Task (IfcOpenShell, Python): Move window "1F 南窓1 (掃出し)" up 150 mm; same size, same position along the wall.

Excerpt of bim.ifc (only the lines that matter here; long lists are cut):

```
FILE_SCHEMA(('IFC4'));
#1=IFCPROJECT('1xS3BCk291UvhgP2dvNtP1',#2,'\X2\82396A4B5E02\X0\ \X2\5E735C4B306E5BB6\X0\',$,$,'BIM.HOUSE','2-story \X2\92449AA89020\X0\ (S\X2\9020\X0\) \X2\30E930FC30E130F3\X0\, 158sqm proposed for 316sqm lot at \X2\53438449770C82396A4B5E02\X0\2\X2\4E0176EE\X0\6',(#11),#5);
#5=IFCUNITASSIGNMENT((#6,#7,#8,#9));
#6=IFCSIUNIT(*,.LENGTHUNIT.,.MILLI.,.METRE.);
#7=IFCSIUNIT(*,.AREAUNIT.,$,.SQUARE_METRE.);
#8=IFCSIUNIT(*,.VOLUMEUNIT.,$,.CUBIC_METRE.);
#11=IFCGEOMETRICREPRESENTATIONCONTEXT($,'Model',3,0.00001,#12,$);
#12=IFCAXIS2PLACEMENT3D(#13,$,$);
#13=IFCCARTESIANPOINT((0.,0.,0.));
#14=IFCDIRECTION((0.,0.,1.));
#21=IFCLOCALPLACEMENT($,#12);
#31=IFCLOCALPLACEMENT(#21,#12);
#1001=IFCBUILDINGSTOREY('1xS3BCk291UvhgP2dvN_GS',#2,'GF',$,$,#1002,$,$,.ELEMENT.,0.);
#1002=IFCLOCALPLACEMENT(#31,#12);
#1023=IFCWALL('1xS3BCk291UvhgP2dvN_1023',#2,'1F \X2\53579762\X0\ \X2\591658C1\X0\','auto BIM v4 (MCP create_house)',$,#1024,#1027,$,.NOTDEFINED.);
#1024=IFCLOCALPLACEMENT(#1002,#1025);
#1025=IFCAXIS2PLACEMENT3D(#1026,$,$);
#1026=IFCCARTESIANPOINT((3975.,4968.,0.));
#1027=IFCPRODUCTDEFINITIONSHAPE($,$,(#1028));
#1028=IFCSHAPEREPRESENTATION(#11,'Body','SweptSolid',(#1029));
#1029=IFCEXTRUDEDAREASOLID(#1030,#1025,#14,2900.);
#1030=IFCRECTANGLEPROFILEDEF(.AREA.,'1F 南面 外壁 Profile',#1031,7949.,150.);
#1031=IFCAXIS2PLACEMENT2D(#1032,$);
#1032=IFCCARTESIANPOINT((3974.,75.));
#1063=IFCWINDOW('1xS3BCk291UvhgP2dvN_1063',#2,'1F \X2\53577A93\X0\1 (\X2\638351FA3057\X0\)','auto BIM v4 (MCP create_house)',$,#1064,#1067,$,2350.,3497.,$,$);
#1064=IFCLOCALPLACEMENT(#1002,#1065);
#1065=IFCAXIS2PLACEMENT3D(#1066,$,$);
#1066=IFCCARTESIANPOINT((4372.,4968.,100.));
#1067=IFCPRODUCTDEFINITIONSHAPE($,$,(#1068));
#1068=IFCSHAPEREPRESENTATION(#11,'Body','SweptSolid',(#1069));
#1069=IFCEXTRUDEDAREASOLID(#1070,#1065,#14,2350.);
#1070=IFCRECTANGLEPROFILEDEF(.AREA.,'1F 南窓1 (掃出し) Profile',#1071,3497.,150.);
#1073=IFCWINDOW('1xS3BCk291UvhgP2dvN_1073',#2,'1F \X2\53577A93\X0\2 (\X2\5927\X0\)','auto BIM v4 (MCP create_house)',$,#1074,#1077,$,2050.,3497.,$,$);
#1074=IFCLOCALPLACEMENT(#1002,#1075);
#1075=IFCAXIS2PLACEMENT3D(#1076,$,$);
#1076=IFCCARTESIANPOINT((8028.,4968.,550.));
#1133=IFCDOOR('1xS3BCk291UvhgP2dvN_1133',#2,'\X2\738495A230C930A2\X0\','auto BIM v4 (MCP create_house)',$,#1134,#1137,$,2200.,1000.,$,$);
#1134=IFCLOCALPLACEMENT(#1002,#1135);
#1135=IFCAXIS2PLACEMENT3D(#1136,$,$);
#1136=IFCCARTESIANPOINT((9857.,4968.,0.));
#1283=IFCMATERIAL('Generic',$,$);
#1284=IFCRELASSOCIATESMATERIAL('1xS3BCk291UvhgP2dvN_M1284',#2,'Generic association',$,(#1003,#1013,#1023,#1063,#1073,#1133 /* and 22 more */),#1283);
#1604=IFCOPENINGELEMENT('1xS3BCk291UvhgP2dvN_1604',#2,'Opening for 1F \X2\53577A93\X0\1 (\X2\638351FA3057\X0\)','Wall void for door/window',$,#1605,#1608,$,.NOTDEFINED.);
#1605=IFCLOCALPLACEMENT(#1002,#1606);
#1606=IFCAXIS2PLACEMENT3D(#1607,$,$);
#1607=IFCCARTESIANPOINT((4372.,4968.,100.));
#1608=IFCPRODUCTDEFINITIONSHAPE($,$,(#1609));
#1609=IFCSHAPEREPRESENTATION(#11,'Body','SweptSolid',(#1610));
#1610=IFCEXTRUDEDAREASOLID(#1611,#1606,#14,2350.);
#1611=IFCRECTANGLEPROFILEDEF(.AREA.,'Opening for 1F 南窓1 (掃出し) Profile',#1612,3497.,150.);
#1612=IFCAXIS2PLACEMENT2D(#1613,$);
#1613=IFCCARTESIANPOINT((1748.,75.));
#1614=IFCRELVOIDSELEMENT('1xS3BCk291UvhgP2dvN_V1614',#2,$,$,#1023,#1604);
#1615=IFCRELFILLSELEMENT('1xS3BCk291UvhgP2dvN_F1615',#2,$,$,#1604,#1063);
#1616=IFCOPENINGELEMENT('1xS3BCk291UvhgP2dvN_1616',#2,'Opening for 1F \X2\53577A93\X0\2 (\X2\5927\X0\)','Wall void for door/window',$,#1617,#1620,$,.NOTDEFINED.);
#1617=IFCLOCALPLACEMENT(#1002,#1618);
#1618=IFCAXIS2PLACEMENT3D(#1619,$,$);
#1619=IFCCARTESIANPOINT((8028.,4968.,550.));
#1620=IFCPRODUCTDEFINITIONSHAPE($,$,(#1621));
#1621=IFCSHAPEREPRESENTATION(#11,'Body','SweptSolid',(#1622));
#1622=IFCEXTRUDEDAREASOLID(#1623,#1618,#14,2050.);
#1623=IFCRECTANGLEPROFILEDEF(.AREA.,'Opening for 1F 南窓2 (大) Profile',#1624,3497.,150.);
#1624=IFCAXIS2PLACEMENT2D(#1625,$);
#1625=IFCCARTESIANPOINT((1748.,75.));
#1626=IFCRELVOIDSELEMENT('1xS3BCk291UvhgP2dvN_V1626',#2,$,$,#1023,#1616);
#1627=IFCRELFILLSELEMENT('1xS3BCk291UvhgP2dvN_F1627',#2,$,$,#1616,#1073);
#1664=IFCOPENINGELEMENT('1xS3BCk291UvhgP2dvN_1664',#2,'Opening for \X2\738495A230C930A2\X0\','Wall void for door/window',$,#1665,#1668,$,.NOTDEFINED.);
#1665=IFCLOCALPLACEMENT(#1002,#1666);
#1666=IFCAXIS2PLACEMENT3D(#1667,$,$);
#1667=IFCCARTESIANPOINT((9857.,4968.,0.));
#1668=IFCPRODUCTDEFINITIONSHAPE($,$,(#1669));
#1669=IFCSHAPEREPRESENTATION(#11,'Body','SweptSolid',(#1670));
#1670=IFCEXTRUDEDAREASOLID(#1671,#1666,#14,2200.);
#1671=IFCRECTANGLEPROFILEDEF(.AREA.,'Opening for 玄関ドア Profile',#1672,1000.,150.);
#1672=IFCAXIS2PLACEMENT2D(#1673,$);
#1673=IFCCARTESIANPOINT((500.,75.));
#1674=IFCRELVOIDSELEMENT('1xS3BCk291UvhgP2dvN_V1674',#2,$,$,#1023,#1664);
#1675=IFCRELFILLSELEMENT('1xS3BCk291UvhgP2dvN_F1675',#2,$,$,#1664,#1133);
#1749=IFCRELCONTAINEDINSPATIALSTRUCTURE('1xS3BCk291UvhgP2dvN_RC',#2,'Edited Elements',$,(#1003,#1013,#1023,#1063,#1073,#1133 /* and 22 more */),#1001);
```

```python
import numpy as np
import ifcopenshell
import ifcopenshell.api.geometry
import ifcopenshell.util.placement
import ifcopenshell.util.unit

model = ifcopenshell.open("bim.ifc")
unit_scale = ifcopenshell.util.unit.calculate_unit_scale(model)

window = model.by_id(1063)
opening = window.FillsVoids[0].RelatingOpeningElement
dz = 0.15 / unit_scale

shift = np.array([0.0, 0.0, dz])
# The window is not placed relative to its opening, so move both.
for product in (opening, window):
    matrix = ifcopenshell.util.placement.get_local_placement(product.ObjectPlacement)
    matrix[:3, 3] += shift
    ifcopenshell.api.geometry.edit_object_placement(model, product=product, matrix=matrix, is_si=False)

print(f"moved by {dz * unit_scale:+.3f} m")

model.write("bim_updated.ifc")
```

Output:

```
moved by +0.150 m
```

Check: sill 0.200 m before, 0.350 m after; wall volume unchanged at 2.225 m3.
